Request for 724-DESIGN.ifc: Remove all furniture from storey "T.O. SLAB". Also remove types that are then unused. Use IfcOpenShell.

First a look at what the model holds.

```python
import ifcopenshell
import ifcopenshell.util.element

model = ifcopenshell.open("724-DESIGN.ifc")
print(model.schema)
storey = next(s for s in model.by_type("IfcBuildingStorey") if s.Name == "T.O. SLAB")
furniture = [e for e in ifcopenshell.util.element.get_decomposition(storey) if e.is_a("IfcFurnishingElement")]
seen = {}
for e in furniture:
    element_type = ifcopenshell.util.element.get_type(e)
    name = element_type.Name if element_type not in (None, e) else None
    seen[name] = seen.get(name, 0) + 1
for name, count in sorted(seen.items(), key=str):
    print(count, "x", name)
```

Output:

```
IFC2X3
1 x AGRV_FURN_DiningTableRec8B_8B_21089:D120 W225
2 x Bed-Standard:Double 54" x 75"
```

```python
import ifcopenshell
import ifcopenshell.api.root
import ifcopenshell.util.element

model = ifcopenshell.open("724-DESIGN.ifc")

storey = next(s for s in model.by_type("IfcBuildingStorey") if s.Name == "T.O. SLAB")
furniture = [e for e in ifcopenshell.util.element.get_decomposition(storey) if e.is_a("IfcFurnishingElement")]
types = {ifcopenshell.util.element.get_type(e) for e in furniture} - {None, *furniture}

for e in furniture:
    ifcopenshell.api.root.remove_product(model, product=e)
print(len(furniture), "removed")

unused = [t for t in types if not ifcopenshell.util.element.get_types(t)]
for t in unused:
    ifcopenshell.api.root.remove_product(model, product=t)
print(len(unused), "unused types removed")

model.write("724-DESIGN_rev.ifc")
```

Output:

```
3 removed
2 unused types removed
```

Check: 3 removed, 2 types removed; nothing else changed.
